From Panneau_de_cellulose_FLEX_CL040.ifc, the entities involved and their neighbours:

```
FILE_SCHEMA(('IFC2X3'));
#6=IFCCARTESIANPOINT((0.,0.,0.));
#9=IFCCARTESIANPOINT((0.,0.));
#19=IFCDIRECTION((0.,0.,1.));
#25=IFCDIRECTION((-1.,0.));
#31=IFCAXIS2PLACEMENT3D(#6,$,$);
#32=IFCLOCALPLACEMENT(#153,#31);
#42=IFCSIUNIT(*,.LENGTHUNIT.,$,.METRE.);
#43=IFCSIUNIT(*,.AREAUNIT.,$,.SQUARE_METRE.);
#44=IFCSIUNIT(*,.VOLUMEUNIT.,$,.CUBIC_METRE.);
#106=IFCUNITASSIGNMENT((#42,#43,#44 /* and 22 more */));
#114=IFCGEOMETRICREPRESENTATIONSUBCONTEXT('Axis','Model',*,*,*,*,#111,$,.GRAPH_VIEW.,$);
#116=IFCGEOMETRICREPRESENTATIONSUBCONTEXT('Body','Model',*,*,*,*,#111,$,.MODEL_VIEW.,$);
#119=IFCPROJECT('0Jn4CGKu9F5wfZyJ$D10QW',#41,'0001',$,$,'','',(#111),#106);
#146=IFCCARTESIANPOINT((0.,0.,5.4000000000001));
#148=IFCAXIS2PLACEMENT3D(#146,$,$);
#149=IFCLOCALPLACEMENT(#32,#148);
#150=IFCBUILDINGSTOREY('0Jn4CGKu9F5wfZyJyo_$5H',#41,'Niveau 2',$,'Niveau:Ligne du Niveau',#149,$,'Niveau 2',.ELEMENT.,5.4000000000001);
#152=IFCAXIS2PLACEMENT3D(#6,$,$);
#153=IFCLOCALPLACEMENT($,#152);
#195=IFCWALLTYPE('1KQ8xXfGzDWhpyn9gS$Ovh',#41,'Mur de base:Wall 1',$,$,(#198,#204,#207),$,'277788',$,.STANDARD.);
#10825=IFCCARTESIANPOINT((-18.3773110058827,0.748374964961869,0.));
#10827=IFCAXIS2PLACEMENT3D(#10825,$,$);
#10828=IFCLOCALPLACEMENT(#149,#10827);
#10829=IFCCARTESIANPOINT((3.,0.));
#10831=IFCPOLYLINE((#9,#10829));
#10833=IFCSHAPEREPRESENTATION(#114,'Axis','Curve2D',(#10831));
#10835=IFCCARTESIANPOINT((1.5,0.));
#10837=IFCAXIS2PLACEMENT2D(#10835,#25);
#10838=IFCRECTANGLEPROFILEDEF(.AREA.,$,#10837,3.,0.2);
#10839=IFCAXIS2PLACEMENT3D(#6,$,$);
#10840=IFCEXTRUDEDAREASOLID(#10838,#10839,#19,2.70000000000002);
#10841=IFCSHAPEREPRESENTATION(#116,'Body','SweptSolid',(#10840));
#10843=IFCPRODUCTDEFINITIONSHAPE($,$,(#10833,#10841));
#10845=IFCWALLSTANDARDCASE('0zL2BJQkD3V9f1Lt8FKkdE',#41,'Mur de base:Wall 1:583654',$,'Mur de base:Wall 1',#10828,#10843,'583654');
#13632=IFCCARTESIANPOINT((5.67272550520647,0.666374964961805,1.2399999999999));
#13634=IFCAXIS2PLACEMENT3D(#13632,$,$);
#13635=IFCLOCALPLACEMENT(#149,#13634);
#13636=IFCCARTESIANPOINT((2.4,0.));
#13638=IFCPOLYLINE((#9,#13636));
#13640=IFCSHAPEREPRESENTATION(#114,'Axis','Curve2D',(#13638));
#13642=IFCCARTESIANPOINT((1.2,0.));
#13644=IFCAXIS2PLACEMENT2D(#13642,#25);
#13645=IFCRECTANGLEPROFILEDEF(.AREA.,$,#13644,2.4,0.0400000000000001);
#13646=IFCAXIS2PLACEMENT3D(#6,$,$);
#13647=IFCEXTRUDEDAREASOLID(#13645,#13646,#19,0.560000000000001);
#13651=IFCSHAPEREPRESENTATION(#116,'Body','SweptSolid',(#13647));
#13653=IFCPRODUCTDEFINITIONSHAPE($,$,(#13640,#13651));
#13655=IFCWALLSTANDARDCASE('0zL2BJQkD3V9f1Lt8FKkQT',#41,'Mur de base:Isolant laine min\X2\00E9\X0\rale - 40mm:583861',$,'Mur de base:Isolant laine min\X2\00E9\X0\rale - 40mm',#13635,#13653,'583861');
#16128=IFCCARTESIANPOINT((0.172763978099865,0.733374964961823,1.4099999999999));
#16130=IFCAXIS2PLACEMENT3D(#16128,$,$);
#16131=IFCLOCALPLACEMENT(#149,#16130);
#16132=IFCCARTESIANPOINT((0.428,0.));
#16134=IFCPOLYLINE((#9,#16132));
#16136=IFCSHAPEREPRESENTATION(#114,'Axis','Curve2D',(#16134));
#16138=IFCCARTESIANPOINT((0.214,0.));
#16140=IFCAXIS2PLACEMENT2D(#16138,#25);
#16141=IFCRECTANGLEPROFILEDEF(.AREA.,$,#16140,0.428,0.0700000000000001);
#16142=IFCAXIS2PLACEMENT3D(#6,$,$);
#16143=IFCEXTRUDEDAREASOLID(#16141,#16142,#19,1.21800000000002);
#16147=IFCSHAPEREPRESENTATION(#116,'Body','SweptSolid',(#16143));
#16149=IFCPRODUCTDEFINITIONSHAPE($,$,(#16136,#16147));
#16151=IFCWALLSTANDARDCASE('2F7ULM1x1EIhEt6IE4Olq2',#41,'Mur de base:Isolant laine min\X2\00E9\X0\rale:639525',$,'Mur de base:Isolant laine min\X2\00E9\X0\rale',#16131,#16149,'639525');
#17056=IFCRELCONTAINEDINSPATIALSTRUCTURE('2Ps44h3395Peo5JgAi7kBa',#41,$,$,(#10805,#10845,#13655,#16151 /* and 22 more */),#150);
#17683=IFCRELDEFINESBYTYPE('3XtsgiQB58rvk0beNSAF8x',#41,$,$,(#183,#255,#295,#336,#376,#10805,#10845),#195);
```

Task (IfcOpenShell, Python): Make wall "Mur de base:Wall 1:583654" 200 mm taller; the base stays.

```python
import ifcopenshell
import ifcopenshell.geom
import ifcopenshell.util.representation
import ifcopenshell.util.shape

model = ifcopenshell.open("Panneau_de_cellulose_FLEX_CL040.ifc")
settings = ifcopenshell.geom.settings()


def volume(element):
    """Net volume in cubic metres, openings subtracted."""
    shape = ifcopenshell.geom.create_shape(settings, element)
    return ifcopenshell.util.shape.get_volume(shape.geometry)


wall = model.by_guid("0zL2BJQkD3V9f1Lt8FKkdE")
before = volume(wall)

body = ifcopenshell.util.representation.get_representation(wall, "Model", "Body")
solid = body.Items[0]
old_height = solid.Depth
solid.Depth += 0.2
after = volume(wall)

print(f"height {old_height:g} -> {solid.Depth:g}, volume {before:.3f} -> {after:.3f} m3")

model.write("Panneau_de_cellulose_FLEX_CL040_updated.ifc")
```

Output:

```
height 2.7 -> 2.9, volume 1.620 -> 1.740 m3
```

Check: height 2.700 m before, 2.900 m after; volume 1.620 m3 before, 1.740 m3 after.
